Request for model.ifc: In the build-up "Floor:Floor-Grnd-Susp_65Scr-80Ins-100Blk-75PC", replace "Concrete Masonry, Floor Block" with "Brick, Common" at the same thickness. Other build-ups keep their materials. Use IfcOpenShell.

First a look at what the model holds.

```python
import ifcopenshell
import ifcopenshell.util.element

model = ifcopenshell.open("model.ifc")
print(model.schema)
for layer_set in model.by_type("IfcMaterialLayerSet"):
    if layer_set.LayerSetName == "Floor:Floor-Grnd-Susp_65Scr-80Ins-100Blk-75PC":
        for layer in layer_set.MaterialLayers:
            print(layer.id(), layer.Material and layer.Material.Name, layer.LayerThickness, sep=" | ")
        print(len(ifcopenshell.util.element.get_elements_by_material(model, layer_set)), "elements and types use it")
print(sorted(m.Name for m in model.by_type("IfcMaterial") if m.Name)[:60])
```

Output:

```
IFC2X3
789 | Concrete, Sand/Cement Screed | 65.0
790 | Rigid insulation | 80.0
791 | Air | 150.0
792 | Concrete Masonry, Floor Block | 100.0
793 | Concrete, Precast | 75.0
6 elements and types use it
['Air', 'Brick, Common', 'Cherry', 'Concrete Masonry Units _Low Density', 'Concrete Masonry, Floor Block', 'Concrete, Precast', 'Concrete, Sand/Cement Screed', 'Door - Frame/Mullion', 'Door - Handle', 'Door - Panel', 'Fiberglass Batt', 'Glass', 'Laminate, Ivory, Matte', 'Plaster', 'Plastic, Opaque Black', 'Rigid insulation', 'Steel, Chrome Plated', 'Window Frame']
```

```python
import ifcopenshell
import ifcopenshell.api.material

model = ifcopenshell.open("model.ifc")

layer_set = next(s for s in model.by_type("IfcMaterialLayerSet") if s.LayerSetName == "Floor:Floor-Grnd-Susp_65Scr-80Ins-100Blk-75PC")
layer = next(l for l in layer_set.MaterialLayers if l.Material and l.Material.Name == "Concrete Masonry, Floor Block")
material = next(m for m in model.by_type("IfcMaterial") if m.Name == "Brick, Common")

# Point this one layer at the other material; renaming the old one would change it everywhere.
ifcopenshell.api.material.edit_layer(model, layer=layer, attributes={}, material=material)

print([l.Material.Name if l.Material else None for l in layer_set.MaterialLayers])

model.write("model_rev.ifc")
```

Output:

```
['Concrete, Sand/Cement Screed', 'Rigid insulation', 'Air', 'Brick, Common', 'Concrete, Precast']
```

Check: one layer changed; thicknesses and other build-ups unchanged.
